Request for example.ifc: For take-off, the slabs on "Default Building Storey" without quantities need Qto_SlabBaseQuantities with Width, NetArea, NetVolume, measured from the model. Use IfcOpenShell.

First a look at what the model holds.

```python
import ifcopenshell
import ifcopenshell.util.element
import ifcopenshell.util.unit

model = ifcopenshell.open("example.ifc")
print(model.schema)
for unit_type in ("LENGTHUNIT", "AREAUNIT", "VOLUMEUNIT"):
    print(unit_type, ifcopenshell.util.unit.calculate_unit_scale(model, unit_type))
storey = next(s for s in model.by_type("IfcBuildingStorey") if s.Name == "Default Building Storey")
slabs = [e for e in ifcopenshell.util.element.get_decomposition(storey) if e.is_a("IfcSlab")]
for e in sorted(slabs, key=lambda e: e.id()):
    print(e.id(), e.is_a(), e.Name, list(ifcopenshell.util.element.get_psets(e, qtos_only=True)), sep=" | ")
```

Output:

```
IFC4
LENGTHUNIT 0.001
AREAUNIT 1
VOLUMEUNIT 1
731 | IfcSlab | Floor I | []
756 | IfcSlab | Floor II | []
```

```python
import ifcopenshell
import ifcopenshell.api.pset
import ifcopenshell.geom
import ifcopenshell.util.element
import ifcopenshell.util.shape
import ifcopenshell.util.unit

model = ifcopenshell.open("example.ifc")
unit_scale = ifcopenshell.util.unit.calculate_unit_scale(model)
area_scale = ifcopenshell.util.unit.calculate_unit_scale(model, "AREAUNIT")
volume_scale = ifcopenshell.util.unit.calculate_unit_scale(model, "VOLUMEUNIT")
settings = ifcopenshell.geom.settings()

storey = next(s for s in model.by_type("IfcBuildingStorey") if s.Name == "Default Building Storey")
slabs = [e for e in ifcopenshell.util.element.get_decomposition(storey) if e.is_a("IfcSlab")]

for e in sorted(slabs, key=lambda e: e.id()):
    if ifcopenshell.util.element.get_psets(e, qtos_only=True, should_inherit=False):
        continue
    # Geometry comes back in metres, in the element's own axes.
    shape = ifcopenshell.geom.create_shape(settings, e)
    values = {
        "Width": ifcopenshell.util.shape.get_z(shape.geometry) / unit_scale,
        "NetArea": ifcopenshell.util.shape.get_footprint_area(shape.geometry) / area_scale,
        "NetVolume": ifcopenshell.util.shape.get_volume(shape.geometry) / volume_scale,
    }
    qto = ifcopenshell.api.pset.add_qto(model, product=e, name="Qto_SlabBaseQuantities")
    ifcopenshell.api.pset.edit_qto(model, qto=qto, properties=values)
    print(e.id(), {k: round(v, 3) for k, v in values.items()})

model.write("example_edited.ifc")
```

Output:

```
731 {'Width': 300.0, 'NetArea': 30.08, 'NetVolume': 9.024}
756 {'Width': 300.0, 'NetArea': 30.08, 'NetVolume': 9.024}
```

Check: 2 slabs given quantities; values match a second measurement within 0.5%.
